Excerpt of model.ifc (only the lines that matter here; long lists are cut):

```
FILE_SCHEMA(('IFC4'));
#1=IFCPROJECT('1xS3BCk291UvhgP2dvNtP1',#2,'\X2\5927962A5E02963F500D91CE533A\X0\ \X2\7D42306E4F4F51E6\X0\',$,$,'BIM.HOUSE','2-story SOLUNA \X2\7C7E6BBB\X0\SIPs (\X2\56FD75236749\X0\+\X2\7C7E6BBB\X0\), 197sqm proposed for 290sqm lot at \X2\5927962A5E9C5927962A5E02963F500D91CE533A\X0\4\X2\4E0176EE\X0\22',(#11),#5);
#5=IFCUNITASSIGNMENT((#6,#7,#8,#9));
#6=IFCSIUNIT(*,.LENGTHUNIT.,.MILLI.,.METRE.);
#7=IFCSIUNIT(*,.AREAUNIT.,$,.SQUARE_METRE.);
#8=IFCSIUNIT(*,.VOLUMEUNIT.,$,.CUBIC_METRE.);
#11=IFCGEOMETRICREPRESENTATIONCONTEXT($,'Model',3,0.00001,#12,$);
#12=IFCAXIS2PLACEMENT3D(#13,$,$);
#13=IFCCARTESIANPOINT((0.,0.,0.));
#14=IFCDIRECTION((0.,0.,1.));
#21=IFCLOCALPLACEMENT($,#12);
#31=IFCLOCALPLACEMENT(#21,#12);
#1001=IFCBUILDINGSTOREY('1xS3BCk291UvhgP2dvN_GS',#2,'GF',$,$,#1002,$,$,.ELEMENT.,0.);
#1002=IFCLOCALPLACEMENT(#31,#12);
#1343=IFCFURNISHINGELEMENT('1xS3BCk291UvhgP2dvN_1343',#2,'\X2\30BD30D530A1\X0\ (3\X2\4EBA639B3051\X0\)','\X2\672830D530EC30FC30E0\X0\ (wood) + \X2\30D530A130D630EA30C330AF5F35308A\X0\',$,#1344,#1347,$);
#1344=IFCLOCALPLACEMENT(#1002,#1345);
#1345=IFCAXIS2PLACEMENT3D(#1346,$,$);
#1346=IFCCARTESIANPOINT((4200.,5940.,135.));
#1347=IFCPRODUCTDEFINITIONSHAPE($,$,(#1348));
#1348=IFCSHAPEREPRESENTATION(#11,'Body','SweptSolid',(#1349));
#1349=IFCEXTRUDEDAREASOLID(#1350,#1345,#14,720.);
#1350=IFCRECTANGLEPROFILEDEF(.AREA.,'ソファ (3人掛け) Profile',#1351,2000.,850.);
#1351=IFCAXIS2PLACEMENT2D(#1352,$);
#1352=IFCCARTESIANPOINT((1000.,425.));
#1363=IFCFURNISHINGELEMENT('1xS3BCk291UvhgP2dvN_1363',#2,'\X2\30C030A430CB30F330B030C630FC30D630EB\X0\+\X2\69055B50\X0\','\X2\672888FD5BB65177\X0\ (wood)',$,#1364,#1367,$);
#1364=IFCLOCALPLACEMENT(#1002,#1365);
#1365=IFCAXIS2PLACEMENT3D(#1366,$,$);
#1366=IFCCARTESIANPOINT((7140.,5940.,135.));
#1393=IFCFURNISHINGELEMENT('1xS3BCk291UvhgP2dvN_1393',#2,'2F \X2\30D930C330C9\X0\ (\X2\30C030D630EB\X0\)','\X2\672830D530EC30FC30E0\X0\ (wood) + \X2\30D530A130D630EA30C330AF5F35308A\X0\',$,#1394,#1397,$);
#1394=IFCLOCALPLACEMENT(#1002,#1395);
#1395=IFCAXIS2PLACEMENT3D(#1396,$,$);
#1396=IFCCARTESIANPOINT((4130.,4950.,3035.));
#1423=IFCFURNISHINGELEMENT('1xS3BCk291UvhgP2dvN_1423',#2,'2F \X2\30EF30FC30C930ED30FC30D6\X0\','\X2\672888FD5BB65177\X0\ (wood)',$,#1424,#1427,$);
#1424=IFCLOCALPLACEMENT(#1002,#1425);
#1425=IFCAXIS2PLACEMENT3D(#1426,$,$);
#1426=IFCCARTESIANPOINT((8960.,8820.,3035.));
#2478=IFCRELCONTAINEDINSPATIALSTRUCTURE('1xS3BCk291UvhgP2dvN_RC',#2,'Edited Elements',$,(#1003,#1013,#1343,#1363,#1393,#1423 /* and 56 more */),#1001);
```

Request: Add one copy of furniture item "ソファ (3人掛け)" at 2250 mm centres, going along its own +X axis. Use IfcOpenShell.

```python
import ifcopenshell
import ifcopenshell.api.geometry
import ifcopenshell.api.root
import ifcopenshell.util.element
import ifcopenshell.util.placement
import ifcopenshell.util.unit

model = ifcopenshell.open("model.ifc")
unit_scale = ifcopenshell.util.unit.calculate_unit_scale(model)


def reuse_history(source, copy):
    """copy_class also copies each property set's owner history, people and application; keep the originals."""
    for rel in copy.IsDefinedBy:
        if rel.is_a("IfcRelDefinesByProperties") and (history := rel.RelatingPropertyDefinition.OwnerHistory):
            rel.RelatingPropertyDefinition.OwnerHistory = source.OwnerHistory
            ifcopenshell.util.element.remove_deep2(model, history)


source = model.by_guid("1xS3BCk291UvhgP2dvN_1343")
base = ifcopenshell.util.placement.get_local_placement(source.ObjectPlacement)
step = base[:3, 0] * 2.25 / unit_scale

for i in range(1, 2):
    copy = ifcopenshell.api.root.copy_class(model, product=source)
    copy.Representation = ifcopenshell.util.element.copy_deep(
        model, source.Representation, exclude=["IfcGeometricRepresentationContext", "IfcRepresentationMap"]
    )
    reuse_history(source, copy)
    matrix = base.copy()
    matrix[:3, 3] += i * step
    print("added at", matrix[:3, 3].round(3) + 0.0)
    ifcopenshell.api.geometry.edit_object_placement(model, product=copy, matrix=matrix, is_si=False)

model.write("model_rev.ifc")
```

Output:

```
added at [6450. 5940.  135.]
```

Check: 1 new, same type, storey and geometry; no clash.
